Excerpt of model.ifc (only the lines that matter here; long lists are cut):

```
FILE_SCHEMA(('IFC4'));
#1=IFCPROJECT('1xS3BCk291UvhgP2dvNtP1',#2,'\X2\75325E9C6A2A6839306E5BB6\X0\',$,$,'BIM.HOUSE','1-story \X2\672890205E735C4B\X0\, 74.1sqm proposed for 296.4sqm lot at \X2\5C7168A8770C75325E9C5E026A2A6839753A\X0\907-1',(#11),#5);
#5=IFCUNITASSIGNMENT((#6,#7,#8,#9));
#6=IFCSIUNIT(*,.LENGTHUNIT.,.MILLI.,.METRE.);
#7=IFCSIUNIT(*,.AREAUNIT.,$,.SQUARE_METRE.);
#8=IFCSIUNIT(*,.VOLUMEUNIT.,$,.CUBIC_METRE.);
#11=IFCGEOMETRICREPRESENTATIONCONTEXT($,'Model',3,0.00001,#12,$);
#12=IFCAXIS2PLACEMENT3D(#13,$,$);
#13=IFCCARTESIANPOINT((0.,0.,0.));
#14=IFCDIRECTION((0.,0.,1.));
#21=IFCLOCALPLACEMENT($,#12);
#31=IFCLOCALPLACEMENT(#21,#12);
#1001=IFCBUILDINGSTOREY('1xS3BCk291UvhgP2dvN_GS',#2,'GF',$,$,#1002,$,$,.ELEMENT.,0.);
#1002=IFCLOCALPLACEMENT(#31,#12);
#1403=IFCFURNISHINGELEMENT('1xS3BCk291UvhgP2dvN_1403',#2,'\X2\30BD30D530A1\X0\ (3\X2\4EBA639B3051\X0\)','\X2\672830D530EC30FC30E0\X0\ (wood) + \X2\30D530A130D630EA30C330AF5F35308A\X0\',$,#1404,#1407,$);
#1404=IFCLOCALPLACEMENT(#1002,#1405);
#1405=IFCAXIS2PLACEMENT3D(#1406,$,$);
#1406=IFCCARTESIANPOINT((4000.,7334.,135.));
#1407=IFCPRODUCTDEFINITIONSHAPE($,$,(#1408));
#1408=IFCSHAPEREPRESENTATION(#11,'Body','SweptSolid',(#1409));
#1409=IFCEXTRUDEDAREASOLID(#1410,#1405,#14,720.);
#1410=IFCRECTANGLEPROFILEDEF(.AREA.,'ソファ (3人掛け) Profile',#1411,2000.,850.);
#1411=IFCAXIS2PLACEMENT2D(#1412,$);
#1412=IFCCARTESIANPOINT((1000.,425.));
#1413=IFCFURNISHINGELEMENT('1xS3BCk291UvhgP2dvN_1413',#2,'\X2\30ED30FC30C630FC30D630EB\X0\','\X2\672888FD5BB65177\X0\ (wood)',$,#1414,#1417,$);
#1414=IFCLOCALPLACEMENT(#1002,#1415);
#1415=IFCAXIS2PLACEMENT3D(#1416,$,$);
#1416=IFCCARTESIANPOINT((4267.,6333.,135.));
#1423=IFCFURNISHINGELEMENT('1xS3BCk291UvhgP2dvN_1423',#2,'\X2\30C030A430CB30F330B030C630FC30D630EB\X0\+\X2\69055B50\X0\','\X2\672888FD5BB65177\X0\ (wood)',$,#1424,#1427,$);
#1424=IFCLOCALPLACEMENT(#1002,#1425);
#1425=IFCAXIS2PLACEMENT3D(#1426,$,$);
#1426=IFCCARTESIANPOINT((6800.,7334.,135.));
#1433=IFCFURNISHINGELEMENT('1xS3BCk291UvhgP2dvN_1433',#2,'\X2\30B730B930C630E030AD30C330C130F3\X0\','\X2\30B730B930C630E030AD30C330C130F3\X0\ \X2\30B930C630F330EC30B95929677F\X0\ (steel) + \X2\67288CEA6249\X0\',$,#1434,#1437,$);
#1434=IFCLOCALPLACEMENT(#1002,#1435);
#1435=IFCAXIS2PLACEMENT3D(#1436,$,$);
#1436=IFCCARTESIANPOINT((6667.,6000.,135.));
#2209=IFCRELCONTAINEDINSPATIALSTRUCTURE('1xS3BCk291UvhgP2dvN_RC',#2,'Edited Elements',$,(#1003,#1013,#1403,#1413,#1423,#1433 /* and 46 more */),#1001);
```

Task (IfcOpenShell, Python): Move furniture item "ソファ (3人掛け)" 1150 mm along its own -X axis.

```python
import ifcopenshell
import ifcopenshell.api.geometry
import ifcopenshell.util.placement

model = ifcopenshell.open("model.ifc")

item = model.by_id(1403)
matrix = ifcopenshell.util.placement.get_local_placement(item.ObjectPlacement)
matrix[:3, 3] -= matrix[:3, 0] * 1150.0
ifcopenshell.api.geometry.edit_object_placement(model, product=item, matrix=matrix, is_si=False)

print(ifcopenshell.util.placement.get_local_placement(item.ObjectPlacement).round(3) + 0.0)

model.write("model-out.ifc")
```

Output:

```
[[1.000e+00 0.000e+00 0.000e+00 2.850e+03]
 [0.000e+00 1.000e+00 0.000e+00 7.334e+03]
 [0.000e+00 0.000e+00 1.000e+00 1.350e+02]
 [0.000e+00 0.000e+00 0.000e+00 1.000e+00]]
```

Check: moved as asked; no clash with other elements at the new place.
